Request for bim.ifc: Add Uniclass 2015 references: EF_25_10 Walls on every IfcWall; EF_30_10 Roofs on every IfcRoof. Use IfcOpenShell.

First a look at what the model holds.

```python
import ifcopenshell

model = ifcopenshell.open("bim.ifc")
print(model.schema)
print("classifications:", [c.Name for c in model.by_type("IfcClassification")])
for ifc_class in ("IfcDoor", "IfcRoof", "IfcStair", "IfcWall", "IfcWindow"):
    print(ifc_class, len(model.by_type(ifc_class)))
```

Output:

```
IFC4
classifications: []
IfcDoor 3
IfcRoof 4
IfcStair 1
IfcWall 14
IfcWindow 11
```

```python
import ifcopenshell
import ifcopenshell.api.classification

model = ifcopenshell.open("bim.ifc")

system = ifcopenshell.api.classification.add_classification(model, classification="Uniclass 2015")

codes = {
    "IfcWall": ("EF_25_10", "Walls"),
    "IfcRoof": ("EF_30_10", "Roofs"),
}
for ifc_class, (code, name) in codes.items():
    products = model.by_type(ifc_class)
    ifcopenshell.api.classification.add_reference(
        model, products=products, classification=system, identification=code, name=name
    )
    print(code, len(products))

model.write("bim_rev.ifc")
```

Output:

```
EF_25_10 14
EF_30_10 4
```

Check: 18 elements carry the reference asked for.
